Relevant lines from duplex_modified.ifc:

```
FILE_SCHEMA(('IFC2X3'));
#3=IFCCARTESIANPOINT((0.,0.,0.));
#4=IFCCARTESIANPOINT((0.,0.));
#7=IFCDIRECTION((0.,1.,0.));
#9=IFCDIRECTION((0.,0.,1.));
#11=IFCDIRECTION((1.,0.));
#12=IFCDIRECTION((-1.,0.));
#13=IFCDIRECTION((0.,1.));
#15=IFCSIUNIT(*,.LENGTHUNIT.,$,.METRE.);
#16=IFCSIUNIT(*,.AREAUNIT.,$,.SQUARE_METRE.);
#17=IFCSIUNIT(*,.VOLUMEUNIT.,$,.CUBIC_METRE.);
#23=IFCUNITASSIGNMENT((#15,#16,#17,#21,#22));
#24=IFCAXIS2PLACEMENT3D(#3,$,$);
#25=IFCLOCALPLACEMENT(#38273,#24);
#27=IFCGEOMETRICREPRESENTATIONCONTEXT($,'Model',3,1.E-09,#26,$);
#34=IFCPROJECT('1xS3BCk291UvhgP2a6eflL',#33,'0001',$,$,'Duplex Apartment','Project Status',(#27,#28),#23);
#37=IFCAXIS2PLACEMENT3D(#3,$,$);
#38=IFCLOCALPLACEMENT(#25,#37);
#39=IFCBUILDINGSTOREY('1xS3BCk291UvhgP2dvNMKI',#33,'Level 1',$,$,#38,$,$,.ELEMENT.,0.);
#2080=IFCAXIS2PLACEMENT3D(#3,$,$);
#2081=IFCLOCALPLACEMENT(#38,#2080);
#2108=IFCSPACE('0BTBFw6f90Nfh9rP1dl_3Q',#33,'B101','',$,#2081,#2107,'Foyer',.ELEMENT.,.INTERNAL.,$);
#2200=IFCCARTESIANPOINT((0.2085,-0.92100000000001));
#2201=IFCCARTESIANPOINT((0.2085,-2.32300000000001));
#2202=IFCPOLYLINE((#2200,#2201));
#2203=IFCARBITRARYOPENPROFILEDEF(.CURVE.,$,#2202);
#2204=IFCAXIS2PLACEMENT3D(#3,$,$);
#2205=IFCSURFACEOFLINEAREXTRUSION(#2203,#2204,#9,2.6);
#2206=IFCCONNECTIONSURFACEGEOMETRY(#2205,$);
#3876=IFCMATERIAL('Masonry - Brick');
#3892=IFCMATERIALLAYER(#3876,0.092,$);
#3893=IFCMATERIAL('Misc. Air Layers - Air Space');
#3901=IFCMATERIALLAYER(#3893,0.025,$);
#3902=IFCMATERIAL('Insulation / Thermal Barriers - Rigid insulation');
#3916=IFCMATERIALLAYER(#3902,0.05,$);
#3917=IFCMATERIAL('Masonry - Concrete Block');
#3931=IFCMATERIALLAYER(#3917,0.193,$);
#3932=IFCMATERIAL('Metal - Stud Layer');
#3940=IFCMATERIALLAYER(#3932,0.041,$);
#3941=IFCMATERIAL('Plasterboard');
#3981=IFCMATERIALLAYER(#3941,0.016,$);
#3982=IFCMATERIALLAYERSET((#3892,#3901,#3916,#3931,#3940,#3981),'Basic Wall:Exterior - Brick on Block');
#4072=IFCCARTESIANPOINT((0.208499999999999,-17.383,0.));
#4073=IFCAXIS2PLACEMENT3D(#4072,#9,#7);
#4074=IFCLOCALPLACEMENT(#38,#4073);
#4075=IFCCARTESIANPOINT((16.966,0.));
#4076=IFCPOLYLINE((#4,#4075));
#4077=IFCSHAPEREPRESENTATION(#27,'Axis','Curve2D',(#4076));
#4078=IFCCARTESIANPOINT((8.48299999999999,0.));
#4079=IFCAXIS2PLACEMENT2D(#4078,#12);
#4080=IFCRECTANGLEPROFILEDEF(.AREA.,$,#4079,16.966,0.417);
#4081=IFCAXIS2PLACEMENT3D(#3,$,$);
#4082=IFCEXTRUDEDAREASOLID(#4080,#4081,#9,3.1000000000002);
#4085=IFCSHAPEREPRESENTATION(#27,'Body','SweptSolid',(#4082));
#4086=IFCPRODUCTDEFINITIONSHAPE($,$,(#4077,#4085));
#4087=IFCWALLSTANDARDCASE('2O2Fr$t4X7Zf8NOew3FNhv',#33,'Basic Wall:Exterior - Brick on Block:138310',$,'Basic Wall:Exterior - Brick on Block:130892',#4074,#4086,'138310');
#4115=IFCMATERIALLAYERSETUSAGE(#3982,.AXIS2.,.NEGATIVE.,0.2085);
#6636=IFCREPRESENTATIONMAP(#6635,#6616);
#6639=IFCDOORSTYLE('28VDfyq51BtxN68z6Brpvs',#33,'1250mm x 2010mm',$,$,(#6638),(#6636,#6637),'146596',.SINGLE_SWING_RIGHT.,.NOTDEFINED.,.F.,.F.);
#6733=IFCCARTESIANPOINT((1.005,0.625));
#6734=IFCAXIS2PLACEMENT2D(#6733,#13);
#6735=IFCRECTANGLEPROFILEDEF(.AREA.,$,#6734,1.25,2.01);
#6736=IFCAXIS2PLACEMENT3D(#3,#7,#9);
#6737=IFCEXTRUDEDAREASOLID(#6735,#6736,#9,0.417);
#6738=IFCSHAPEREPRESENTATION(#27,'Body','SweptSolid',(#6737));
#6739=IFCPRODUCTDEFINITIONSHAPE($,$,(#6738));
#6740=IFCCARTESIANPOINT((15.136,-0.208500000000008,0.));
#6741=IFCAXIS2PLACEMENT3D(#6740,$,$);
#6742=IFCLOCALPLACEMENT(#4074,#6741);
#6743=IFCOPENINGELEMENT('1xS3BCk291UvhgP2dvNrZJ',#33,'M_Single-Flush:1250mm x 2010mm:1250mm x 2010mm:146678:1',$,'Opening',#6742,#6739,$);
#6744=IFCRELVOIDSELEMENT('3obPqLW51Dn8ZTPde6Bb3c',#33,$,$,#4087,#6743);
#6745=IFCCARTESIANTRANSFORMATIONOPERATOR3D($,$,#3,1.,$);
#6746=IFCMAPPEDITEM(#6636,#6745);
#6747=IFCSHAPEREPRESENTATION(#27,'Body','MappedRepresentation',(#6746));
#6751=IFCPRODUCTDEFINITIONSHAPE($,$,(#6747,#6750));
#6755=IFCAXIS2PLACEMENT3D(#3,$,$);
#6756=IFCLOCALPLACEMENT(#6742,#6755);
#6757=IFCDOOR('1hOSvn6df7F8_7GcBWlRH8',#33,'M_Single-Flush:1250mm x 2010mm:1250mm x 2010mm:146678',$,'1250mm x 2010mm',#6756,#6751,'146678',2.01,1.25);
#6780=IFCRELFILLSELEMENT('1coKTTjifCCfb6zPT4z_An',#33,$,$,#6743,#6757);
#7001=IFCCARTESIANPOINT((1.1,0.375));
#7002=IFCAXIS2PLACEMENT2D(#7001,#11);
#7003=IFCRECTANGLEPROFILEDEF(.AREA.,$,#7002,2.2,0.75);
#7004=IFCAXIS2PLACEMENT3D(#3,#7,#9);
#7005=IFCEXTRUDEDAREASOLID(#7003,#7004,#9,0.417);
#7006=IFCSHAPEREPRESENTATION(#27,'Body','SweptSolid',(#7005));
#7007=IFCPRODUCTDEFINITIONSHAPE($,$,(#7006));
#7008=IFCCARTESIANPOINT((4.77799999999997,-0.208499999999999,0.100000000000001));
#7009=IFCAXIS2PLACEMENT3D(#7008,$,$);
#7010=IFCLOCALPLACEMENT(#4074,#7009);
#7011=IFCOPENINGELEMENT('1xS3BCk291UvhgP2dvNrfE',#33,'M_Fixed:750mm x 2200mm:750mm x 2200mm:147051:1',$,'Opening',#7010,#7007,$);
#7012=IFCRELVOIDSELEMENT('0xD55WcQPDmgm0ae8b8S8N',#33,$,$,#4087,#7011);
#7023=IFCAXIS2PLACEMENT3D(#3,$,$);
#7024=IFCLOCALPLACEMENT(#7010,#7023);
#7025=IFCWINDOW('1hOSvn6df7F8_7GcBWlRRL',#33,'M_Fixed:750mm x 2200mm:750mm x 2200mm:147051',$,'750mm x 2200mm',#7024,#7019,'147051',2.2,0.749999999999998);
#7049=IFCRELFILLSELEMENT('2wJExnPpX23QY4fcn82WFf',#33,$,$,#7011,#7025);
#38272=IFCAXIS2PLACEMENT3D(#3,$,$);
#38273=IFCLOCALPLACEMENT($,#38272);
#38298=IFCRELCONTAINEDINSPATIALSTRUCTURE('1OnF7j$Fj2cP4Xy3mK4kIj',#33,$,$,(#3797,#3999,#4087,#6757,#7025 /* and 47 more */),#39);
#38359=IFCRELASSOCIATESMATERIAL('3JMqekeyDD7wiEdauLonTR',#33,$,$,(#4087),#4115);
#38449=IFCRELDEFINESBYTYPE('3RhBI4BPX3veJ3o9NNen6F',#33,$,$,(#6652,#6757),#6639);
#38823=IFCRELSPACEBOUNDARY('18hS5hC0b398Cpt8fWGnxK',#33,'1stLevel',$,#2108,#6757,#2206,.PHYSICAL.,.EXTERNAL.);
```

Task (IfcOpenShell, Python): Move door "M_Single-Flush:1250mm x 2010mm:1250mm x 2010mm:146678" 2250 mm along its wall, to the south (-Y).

```python
import numpy as np
import ifcopenshell
import ifcopenshell.api.geometry
import ifcopenshell.util.placement
import ifcopenshell.util.unit

model = ifcopenshell.open("duplex_modified.ifc")
unit_scale = ifcopenshell.util.unit.calculate_unit_scale(model)

door = model.by_guid("1hOSvn6df7F8_7GcBWlRH8")
opening = door.FillsVoids[0].RelatingOpeningElement
wall = opening.VoidsElements[0].RelatingBuildingElement

wall_matrix = ifcopenshell.util.placement.get_local_placement(wall.ObjectPlacement)
shift = wall_matrix[:3, 0] * -2.25 / unit_scale
before = ifcopenshell.util.placement.get_local_placement(door.ObjectPlacement)[:3, 3].copy()

# The door is placed relative to its opening, so it follows when the opening moves.
matrix = ifcopenshell.util.placement.get_local_placement(opening.ObjectPlacement)
matrix[:3, 3] += shift
ifcopenshell.api.geometry.edit_object_placement(
    model, product=opening, matrix=matrix, is_si=False, should_transform_children=True
)

# Space boundary surfaces are stored in each space's coordinates; move them too.
for rel in door.ProvidesBoundaries:
    if not rel.ConnectionGeometry:
        continue
    surface = rel.ConnectionGeometry.SurfaceOnRelatingElement
    space_matrix = ifcopenshell.util.placement.get_local_placement(rel.RelatingSpace.ObjectPlacement)
    point = np.array(surface.Position.Location.Coordinates) + space_matrix[:3, :3].T @ shift
    surface.Position = model.createIfcAxis2Placement3D(
        model.createIfcCartesianPoint(point.tolist()), surface.Position.Axis, surface.Position.RefDirection
    )

after = ifcopenshell.util.placement.get_local_placement(door.ObjectPlacement)[:3, 3]
print("door moved by", (after - before).round(3) + 0.0)

model.write("duplex_modified-out.ifc")
```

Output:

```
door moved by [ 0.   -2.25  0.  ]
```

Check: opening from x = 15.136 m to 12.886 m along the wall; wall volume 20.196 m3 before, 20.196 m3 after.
